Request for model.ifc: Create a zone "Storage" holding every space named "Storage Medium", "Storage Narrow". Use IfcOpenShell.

First a look at what the model holds.

```python
import ifcopenshell

model = ifcopenshell.open("model.ifc")
print(model.schema)
seen = {}
for space in model.by_type("IfcSpace"):
    seen[space.LongName] = seen.get(space.LongName, 0) + 1
for name, count in sorted(seen.items(), key=str):
    print(count, "x", name)
print("zones:", [z.Name for z in model.by_type("IfcZone")][:20])
```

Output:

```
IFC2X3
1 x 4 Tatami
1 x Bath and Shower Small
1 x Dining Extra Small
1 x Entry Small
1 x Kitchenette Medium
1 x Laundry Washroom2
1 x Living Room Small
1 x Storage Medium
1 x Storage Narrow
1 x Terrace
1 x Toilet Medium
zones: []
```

```python
import ifcopenshell
import ifcopenshell.api.group
import ifcopenshell.api.root

model = ifcopenshell.open("model.ifc")

names = {"Storage Medium", "Storage Narrow"}
spaces = [s for s in model.by_type("IfcSpace") if s.LongName in names]

zone = ifcopenshell.api.root.create_entity(model, ifc_class="IfcZone", name="Storage")
ifcopenshell.api.group.assign_group(model, products=spaces, group=zone)
print(len(spaces), "spaces in", zone.Name)

model.write("model_edited.ifc")
```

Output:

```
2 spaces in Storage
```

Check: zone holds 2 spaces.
